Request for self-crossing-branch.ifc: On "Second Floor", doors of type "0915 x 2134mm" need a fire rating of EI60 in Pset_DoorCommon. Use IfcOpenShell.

First a look at what the model holds.

```python
import ifcopenshell
import ifcopenshell.util.element

model = ifcopenshell.open("self-crossing-branch.ifc")
print(model.schema)
storey = next(s for s in model.by_type("IfcBuildingStorey") if s.Name == "Second Floor")
doors = [e for e in ifcopenshell.util.element.get_decomposition(storey) if e.is_a("IfcDoor")]
seen = {}
for e in doors:
    element_type = ifcopenshell.util.element.get_type(e)
    key = (element_type.Name if element_type != e and element_type else None, ifcopenshell.util.element.get_pset(e, "Pset_DoorCommon", "FireRating"))
    seen[key] = seen.get(key, 0) + 1
for (name, value), count in sorted(seen.items(), key=str):
    print(count, "x", name, "|", value)
```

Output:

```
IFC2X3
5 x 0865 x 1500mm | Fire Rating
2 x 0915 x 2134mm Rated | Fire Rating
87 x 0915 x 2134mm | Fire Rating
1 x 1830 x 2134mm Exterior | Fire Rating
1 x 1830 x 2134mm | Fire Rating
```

```python
import ifcopenshell
import ifcopenshell.api.pset
import ifcopenshell.util.element

model = ifcopenshell.open("self-crossing-branch.ifc")

storey = next(s for s in model.by_type("IfcBuildingStorey") if s.Name == "Second Floor")
doors = [e for e in ifcopenshell.util.element.get_decomposition(storey) if e.is_a("IfcDoor")]

count = 0
for e in doors:
    element_type = ifcopenshell.util.element.get_type(e)
    if element_type in (None, e) or element_type.Name != "0915 x 2134mm":
        continue
    # add_pset returns the element's existing set when there is one.
    pset = ifcopenshell.api.pset.add_pset(model, product=e, name="Pset_DoorCommon")
    ifcopenshell.api.pset.edit_pset(model, pset=pset, properties={"FireRating": "EI60"})
    count += 1

print(count, "doors updated")

model.write("self-crossing-branch_edited.ifc")
```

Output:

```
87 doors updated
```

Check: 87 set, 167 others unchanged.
